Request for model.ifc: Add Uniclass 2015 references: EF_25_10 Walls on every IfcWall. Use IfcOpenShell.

First a look at what the model holds.

```python
import ifcopenshell

model = ifcopenshell.open("model.ifc")
print(model.schema)
print("classifications:", [c.Name for c in model.by_type("IfcClassification")])
for ifc_class in ("IfcDoor", "IfcRoof", "IfcStair", "IfcWall", "IfcWindow"):
    print(ifc_class, len(model.by_type(ifc_class)))
```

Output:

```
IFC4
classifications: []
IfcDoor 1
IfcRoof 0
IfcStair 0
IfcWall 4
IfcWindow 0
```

```python
import ifcopenshell
import ifcopenshell.api.classification

model = ifcopenshell.open("model.ifc")

system = ifcopenshell.api.classification.add_classification(model, classification="Uniclass 2015")

codes = {
    "IfcWall": ("EF_25_10", "Walls"),
}
for ifc_class, (code, name) in codes.items():
    products = model.by_type(ifc_class)
    ifcopenshell.api.classification.add_reference(
        model, products=products, classification=system, identification=code, name=name
    )
    print(code, len(products))

model.write("model_edited.ifc")
```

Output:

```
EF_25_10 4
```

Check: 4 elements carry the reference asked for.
